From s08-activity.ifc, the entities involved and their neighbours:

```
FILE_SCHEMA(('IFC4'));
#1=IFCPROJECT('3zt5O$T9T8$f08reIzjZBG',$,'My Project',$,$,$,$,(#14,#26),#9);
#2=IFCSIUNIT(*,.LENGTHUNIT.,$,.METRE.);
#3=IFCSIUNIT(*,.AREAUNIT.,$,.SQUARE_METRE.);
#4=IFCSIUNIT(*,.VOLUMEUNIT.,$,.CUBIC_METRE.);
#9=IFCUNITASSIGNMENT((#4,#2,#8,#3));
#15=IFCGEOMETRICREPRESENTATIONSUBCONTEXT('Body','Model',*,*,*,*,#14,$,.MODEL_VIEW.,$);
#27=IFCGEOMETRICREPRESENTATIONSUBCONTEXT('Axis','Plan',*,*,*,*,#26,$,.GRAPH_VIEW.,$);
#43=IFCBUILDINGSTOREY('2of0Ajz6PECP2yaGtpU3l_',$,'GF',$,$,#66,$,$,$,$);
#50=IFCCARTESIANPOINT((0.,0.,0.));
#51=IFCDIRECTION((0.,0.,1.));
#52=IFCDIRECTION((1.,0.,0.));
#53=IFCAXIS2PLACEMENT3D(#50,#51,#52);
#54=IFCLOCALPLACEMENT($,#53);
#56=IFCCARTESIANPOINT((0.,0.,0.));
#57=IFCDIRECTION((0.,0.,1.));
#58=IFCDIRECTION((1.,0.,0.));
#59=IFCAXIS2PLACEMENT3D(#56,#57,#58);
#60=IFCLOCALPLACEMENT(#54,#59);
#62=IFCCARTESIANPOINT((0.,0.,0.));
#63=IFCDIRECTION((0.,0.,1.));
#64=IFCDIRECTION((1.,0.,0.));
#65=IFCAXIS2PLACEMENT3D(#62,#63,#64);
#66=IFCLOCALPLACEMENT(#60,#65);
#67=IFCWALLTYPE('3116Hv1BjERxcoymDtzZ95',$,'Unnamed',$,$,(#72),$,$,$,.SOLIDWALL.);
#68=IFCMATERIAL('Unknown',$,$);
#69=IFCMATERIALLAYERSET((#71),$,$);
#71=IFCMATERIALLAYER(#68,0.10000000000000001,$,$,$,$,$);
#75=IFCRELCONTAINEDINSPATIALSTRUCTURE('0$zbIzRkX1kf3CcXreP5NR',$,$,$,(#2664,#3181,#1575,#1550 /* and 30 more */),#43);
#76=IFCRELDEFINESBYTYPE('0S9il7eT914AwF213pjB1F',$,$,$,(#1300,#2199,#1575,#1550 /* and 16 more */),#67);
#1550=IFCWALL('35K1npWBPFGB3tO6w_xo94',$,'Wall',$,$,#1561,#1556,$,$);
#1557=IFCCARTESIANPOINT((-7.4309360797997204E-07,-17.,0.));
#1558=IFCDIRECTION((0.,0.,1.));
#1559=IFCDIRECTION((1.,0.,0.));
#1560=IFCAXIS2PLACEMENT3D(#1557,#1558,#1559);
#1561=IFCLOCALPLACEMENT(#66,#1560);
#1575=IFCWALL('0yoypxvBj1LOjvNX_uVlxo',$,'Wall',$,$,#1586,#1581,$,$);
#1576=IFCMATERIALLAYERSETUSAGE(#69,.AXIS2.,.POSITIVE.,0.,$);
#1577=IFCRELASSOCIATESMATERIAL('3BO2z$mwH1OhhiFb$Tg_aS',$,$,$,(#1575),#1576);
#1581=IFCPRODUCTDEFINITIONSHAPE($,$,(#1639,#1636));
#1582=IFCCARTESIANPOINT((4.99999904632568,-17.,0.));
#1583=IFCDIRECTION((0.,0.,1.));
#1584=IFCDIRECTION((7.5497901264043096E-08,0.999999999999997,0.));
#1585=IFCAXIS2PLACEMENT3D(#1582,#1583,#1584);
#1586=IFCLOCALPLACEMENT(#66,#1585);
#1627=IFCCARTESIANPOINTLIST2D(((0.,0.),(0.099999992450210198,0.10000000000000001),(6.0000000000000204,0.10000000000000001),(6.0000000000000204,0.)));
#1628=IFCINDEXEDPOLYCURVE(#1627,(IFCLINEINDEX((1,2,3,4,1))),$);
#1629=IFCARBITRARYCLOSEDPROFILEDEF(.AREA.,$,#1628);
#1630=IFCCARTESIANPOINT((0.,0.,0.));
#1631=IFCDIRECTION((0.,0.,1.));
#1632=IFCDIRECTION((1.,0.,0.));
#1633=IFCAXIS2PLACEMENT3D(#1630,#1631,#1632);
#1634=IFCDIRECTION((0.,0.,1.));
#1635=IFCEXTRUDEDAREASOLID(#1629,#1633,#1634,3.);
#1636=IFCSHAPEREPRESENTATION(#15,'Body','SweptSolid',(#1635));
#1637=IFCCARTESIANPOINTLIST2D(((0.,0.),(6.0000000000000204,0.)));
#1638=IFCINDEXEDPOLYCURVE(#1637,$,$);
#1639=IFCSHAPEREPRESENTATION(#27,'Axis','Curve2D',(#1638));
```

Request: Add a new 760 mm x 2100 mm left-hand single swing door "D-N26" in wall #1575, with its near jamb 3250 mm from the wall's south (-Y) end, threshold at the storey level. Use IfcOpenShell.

```python
import numpy as np
import ifcopenshell
import ifcopenshell.api.feature
import ifcopenshell.api.geometry
import ifcopenshell.api.root
import ifcopenshell.api.spatial
import ifcopenshell.geom
import ifcopenshell.util.element
import ifcopenshell.util.placement
import ifcopenshell.util.representation
import ifcopenshell.util.shape
import ifcopenshell.util.unit

model = ifcopenshell.open("s08-activity.ifc")
unit_scale = ifcopenshell.util.unit.calculate_unit_scale(model)
settings = ifcopenshell.geom.settings()


def volume(element):
    """Net volume in cubic metres, openings subtracted."""
    shape = ifcopenshell.geom.create_shape(settings, element)
    return ifcopenshell.util.shape.get_volume(shape.geometry)


wall = model.by_guid("0yoypxvBj1LOjvNX_uVlxo")
storey = ifcopenshell.util.element.get_container(wall, ifc_class="IfcBuildingStorey")
context = ifcopenshell.util.representation.get_context(model, "Model", "Body", "MODEL_VIEW")
before = volume(wall)

width, height, from_end, sill = 0.76, 2.1, 3.25, 0.0  # metres

# The wall runs along its own X axis, and the end named is its -X end.
wall_shape = ifcopenshell.geom.create_shape(settings, wall)
x, y, z = ifcopenshell.util.shape.get_vertices(wall_shape.geometry).T
start = x.min() + from_end
face, thickness = float(y.min()), float(y.max() - y.min())
wall_matrix = ifcopenshell.util.placement.get_local_placement(wall.ObjectPlacement)
level = ifcopenshell.util.placement.get_local_placement(storey.ObjectPlacement)[2, 3]


def in_wall(x, y):
    """Placement at x, y metres in the wall's axes, at sill height."""
    matrix = wall_matrix.copy()
    matrix[:, 3] = wall_matrix @ np.array([x / unit_scale, y / unit_scale, 0.0, 1.0])
    matrix[2, 3] = level + sill / unit_scale
    return matrix


# Opening: a box that overshoots both wall faces by 50 mm.
opening = ifcopenshell.api.root.create_entity(model, ifc_class="IfcOpeningElement", predefined_type="OPENING")
box = ifcopenshell.api.geometry.add_wall_representation(
    model, context=context, length=width, height=height, thickness=thickness + 0.1
)
ifcopenshell.api.geometry.assign_representation(model, product=opening, representation=box)
ifcopenshell.api.geometry.edit_object_placement(model, product=opening, matrix=in_wall(start, face - 0.05), is_si=False)
ifcopenshell.api.feature.add_feature(model, feature=opening, element=wall)

door = ifcopenshell.api.root.create_entity(model, ifc_class="IfcDoor", name="D-N26", predefined_type="DOOR")
door.OverallWidth, door.OverallHeight = width / unit_scale, height / unit_scale
door.OperationType = "SINGLE_SWING_LEFT"
body = ifcopenshell.api.geometry.add_door_representation(
    model,
    context=context,
    overall_width=door.OverallWidth,
    overall_height=door.OverallHeight,
    operation_type="SINGLE_SWING_LEFT",
    lining_properties={"LiningDepth": thickness / unit_scale, "ThresholdDepth": thickness / unit_scale},
)
ifcopenshell.api.geometry.assign_representation(model, product=door, representation=body)
ifcopenshell.api.spatial.assign_container(model, products=[door], relating_structure=storey)
ifcopenshell.api.feature.add_filling(model, opening=opening, element=door)

# The lining spans the wall, so the door starts at the wall face.
ifcopenshell.api.geometry.edit_object_placement(model, product=door, matrix=in_wall(start, face), is_si=False)

after = volume(wall)

print(f"wall volume {before:.3f} -> {after:.3f} m3")

model.write("s08-activity-out.ifc")
```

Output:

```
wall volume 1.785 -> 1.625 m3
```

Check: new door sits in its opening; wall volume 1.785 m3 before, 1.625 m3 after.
